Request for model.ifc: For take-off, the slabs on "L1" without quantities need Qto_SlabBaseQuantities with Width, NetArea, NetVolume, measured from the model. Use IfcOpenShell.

First a look at what the model holds.

```python
import ifcopenshell
import ifcopenshell.util.element
import ifcopenshell.util.unit

model = ifcopenshell.open("model.ifc")
print(model.schema)
for unit_type in ("LENGTHUNIT", "AREAUNIT", "VOLUMEUNIT"):
    print(unit_type, ifcopenshell.util.unit.calculate_unit_scale(model, unit_type))
storey = next(s for s in model.by_type("IfcBuildingStorey") if s.Name == "L1")
slabs = [e for e in ifcopenshell.util.element.get_decomposition(storey) if e.is_a("IfcSlab")]
for e in sorted(slabs, key=lambda e: e.id()):
    print(e.id(), e.is_a(), e.Name, list(ifcopenshell.util.element.get_psets(e, qtos_only=True)), sep=" | ")
```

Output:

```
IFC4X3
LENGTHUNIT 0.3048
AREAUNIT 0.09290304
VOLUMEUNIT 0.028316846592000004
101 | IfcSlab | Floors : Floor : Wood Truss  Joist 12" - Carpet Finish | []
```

```python
import ifcopenshell
import ifcopenshell.api.pset
import ifcopenshell.geom
import ifcopenshell.util.element
import ifcopenshell.util.shape
import ifcopenshell.util.unit

model = ifcopenshell.open("model.ifc")
unit_scale = ifcopenshell.util.unit.calculate_unit_scale(model)
area_scale = ifcopenshell.util.unit.calculate_unit_scale(model, "AREAUNIT")
volume_scale = ifcopenshell.util.unit.calculate_unit_scale(model, "VOLUMEUNIT")
settings = ifcopenshell.geom.settings()

storey = next(s for s in model.by_type("IfcBuildingStorey") if s.Name == "L1")
slabs = [e for e in ifcopenshell.util.element.get_decomposition(storey) if e.is_a("IfcSlab")]

for e in sorted(slabs, key=lambda e: e.id()):
    if ifcopenshell.util.element.get_psets(e, qtos_only=True, should_inherit=False):
        continue
    # Geometry comes back in metres, in the element's own axes.
    shape = ifcopenshell.geom.create_shape(settings, e)
    values = {
        "Width": ifcopenshell.util.shape.get_z(shape.geometry) / unit_scale,
        "NetArea": ifcopenshell.util.shape.get_footprint_area(shape.geometry) / area_scale,
        "NetVolume": ifcopenshell.util.shape.get_volume(shape.geometry) / volume_scale,
    }
    qto = ifcopenshell.api.pset.add_qto(model, product=e, name="Qto_SlabBaseQuantities")
    ifcopenshell.api.pset.edit_qto(model, qto=qto, properties=values)
    print(e.id(), {k: round(v, 3) for k, v in values.items()})

model.write("model_v2.ifc")
```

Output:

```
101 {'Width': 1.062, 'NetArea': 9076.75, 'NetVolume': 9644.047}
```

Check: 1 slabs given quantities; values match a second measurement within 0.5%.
